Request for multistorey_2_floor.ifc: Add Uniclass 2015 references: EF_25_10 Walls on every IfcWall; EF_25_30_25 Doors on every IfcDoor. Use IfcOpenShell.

First a look at what the model holds.

```python
import ifcopenshell

model = ifcopenshell.open("multistorey_2_floor.ifc")
print(model.schema)
print("classifications:", [c.Name for c in model.by_type("IfcClassification")])
for ifc_class in ("IfcDoor", "IfcRoof", "IfcStair", "IfcWall", "IfcWindow"):
    print(ifc_class, len(model.by_type(ifc_class)))
```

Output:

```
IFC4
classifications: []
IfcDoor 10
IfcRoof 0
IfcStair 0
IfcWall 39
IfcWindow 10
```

```python
import ifcopenshell
import ifcopenshell.api.classification

model = ifcopenshell.open("multistorey_2_floor.ifc")

system = ifcopenshell.api.classification.add_classification(model, classification="Uniclass 2015")

codes = {
    "IfcWall": ("EF_25_10", "Walls"),
    "IfcDoor": ("EF_25_30_25", "Doors"),
}
for ifc_class, (code, name) in codes.items():
    products = model.by_type(ifc_class)
    ifcopenshell.api.classification.add_reference(
        model, products=products, classification=system, identification=code, name=name
    )
    print(code, len(products))

model.write("multistorey_2_floor_updated.ifc")
```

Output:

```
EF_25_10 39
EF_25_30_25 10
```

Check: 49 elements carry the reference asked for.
